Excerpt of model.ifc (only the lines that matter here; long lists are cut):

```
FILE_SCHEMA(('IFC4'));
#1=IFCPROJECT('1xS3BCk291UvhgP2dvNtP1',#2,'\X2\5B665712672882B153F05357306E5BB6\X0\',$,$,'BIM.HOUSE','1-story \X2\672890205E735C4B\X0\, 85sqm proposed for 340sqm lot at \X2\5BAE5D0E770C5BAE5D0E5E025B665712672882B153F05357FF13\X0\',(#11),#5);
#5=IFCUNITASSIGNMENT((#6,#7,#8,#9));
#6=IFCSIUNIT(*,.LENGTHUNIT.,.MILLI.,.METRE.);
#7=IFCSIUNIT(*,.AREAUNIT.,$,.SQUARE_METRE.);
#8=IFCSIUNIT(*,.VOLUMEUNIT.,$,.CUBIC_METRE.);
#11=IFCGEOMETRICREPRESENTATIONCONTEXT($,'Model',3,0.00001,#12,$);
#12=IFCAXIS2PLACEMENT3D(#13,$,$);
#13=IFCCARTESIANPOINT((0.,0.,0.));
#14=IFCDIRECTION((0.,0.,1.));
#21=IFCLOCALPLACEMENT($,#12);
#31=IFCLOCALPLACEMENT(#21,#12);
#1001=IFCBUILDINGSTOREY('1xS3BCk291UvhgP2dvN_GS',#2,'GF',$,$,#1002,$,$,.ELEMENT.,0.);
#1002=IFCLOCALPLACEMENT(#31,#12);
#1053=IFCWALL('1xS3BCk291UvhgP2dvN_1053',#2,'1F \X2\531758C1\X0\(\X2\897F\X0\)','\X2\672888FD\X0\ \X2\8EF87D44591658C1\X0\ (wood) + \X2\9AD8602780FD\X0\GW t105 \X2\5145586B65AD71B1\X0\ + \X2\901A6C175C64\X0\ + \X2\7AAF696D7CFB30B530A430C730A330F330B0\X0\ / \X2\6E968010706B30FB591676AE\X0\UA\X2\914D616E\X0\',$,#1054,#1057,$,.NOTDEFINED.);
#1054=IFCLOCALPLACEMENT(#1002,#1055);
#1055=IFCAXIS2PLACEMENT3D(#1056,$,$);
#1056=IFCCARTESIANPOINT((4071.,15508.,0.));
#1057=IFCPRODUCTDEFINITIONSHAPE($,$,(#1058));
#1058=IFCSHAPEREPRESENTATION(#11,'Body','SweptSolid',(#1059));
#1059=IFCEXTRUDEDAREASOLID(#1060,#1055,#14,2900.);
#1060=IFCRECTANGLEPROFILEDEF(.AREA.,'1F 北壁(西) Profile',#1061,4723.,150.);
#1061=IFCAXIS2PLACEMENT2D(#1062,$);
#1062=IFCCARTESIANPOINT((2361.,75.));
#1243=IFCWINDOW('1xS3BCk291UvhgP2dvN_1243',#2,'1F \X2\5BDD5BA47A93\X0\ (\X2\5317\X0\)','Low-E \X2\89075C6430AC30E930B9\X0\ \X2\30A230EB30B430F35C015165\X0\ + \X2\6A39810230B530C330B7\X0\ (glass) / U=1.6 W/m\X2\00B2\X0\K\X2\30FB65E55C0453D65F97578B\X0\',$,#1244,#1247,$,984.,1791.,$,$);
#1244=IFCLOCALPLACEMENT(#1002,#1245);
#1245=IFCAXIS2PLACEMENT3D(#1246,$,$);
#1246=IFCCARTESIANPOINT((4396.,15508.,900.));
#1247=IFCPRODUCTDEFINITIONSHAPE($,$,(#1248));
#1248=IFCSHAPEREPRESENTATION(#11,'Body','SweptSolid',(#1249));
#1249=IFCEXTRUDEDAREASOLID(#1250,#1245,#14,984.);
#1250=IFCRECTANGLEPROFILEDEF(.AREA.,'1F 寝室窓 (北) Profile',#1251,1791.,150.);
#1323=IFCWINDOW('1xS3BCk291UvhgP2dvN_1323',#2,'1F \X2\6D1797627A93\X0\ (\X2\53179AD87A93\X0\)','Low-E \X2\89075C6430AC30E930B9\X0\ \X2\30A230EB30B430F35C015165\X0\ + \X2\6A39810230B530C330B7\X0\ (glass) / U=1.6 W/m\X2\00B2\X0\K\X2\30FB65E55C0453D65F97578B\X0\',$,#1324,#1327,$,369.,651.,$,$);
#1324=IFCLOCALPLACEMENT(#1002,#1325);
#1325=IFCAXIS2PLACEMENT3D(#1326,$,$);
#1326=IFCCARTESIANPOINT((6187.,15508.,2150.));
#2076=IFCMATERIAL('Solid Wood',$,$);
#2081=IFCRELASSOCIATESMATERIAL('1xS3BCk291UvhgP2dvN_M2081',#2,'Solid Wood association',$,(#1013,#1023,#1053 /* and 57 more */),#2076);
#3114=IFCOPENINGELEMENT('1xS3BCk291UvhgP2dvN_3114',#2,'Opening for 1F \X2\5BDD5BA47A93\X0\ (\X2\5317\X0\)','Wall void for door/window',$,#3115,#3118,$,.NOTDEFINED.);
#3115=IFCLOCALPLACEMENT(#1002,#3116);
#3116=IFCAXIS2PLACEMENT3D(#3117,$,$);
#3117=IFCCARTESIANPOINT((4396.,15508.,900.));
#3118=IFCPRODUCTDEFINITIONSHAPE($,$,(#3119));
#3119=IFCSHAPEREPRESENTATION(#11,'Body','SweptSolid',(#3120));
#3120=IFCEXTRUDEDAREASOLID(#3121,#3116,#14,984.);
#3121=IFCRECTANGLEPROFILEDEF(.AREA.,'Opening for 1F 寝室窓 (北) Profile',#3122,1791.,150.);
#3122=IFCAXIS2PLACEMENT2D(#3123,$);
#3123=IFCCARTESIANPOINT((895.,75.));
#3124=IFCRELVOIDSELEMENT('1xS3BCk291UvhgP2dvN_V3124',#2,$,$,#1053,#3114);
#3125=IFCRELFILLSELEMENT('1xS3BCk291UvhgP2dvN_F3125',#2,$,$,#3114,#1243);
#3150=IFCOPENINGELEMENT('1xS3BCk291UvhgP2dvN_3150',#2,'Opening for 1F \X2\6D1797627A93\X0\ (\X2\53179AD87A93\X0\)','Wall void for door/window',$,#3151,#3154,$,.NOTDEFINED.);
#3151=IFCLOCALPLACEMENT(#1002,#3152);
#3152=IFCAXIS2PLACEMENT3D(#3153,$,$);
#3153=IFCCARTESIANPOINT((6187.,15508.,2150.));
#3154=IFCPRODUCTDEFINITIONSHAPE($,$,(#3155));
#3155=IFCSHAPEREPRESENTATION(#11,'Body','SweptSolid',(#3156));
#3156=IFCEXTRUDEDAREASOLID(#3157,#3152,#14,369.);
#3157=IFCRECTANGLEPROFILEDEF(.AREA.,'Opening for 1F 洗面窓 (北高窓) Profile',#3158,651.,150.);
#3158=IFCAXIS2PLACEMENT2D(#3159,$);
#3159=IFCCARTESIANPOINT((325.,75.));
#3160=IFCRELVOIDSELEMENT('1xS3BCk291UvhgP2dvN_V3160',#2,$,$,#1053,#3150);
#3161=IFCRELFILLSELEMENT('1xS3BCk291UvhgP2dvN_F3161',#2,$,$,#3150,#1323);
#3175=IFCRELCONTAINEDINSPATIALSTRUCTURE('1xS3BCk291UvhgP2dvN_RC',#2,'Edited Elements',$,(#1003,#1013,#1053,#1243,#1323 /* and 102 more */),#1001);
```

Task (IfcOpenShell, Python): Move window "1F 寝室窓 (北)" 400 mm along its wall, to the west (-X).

```python
import ifcopenshell
import ifcopenshell.api.geometry
import ifcopenshell.util.placement

model = ifcopenshell.open("model.ifc")

window = model.by_guid("1xS3BCk291UvhgP2dvN_1243")
opening = window.FillsVoids[0].RelatingOpeningElement
wall = opening.VoidsElements[0].RelatingBuildingElement

wall_matrix = ifcopenshell.util.placement.get_local_placement(wall.ObjectPlacement)
shift = wall_matrix[:3, 0] * -400.0
before = ifcopenshell.util.placement.get_local_placement(window.ObjectPlacement)[:3, 3].copy()

# The window is not placed relative to its opening, so move both.
for product in (opening, window):
    matrix = ifcopenshell.util.placement.get_local_placement(product.ObjectPlacement)
    matrix[:3, 3] += shift
    ifcopenshell.api.geometry.edit_object_placement(model, product=product, matrix=matrix, is_si=False)

after = ifcopenshell.util.placement.get_local_placement(window.ObjectPlacement)[:3, 3]
print("window moved by", (after - before).round(3) + 0.0)

model.write("model_edited.ifc")
```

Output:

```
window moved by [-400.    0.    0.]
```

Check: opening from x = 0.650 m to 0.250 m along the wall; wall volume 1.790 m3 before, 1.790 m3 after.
